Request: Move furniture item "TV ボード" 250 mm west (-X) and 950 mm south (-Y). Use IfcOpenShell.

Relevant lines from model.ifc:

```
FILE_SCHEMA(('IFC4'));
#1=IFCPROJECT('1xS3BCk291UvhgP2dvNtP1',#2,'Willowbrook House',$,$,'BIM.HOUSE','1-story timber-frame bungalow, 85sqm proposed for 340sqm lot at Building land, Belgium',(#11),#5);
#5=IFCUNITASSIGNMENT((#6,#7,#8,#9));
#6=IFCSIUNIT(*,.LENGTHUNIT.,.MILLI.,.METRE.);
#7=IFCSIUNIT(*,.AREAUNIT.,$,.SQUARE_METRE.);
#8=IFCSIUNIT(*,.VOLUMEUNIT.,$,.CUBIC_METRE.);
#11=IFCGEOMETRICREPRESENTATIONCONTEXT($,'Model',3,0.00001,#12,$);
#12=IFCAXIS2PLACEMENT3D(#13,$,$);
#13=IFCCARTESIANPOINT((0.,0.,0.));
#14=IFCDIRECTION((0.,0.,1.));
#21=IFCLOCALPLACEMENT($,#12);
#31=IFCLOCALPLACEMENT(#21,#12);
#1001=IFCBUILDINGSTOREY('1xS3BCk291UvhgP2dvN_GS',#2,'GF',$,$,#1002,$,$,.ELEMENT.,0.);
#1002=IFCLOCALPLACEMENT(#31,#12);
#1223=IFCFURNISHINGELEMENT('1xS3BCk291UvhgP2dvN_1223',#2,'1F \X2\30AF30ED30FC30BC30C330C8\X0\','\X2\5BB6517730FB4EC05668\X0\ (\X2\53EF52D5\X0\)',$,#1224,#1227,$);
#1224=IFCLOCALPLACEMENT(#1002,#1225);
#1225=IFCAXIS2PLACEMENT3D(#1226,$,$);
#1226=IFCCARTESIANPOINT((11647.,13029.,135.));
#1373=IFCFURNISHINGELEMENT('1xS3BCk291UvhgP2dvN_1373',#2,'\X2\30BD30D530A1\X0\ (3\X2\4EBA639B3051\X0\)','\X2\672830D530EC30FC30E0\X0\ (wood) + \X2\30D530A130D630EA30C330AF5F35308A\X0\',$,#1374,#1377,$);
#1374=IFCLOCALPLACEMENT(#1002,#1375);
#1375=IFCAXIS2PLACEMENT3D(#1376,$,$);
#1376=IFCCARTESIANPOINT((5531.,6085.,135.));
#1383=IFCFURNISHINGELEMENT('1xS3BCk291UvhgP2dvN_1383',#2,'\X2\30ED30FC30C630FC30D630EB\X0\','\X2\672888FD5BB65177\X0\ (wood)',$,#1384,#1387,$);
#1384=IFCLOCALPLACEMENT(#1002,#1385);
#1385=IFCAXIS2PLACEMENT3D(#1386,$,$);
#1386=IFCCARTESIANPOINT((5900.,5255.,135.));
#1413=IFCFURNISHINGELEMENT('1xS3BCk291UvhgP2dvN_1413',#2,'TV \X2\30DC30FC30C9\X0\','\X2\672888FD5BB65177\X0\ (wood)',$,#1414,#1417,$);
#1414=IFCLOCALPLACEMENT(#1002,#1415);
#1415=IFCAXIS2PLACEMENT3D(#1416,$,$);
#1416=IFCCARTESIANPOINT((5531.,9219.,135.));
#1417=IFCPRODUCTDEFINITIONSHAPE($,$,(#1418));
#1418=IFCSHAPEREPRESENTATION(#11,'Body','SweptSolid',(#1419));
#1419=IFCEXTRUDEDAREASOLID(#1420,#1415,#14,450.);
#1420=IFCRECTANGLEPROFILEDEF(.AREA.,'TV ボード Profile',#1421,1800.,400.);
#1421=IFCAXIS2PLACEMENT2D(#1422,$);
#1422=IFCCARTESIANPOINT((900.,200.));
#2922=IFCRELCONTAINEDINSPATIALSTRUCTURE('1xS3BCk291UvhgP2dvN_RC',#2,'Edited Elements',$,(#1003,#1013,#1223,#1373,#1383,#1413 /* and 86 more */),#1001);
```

```python
import ifcopenshell
import ifcopenshell.api.geometry
import ifcopenshell.util.placement

model = ifcopenshell.open("model.ifc")

item = model.by_id(1413)
matrix = ifcopenshell.util.placement.get_local_placement(item.ObjectPlacement)
matrix[0, 3] -= 250.0
matrix[1, 3] -= 950.0
ifcopenshell.api.geometry.edit_object_placement(model, product=item, matrix=matrix, is_si=False)

print(ifcopenshell.util.placement.get_local_placement(item.ObjectPlacement).round(3) + 0.0)

model.write("model_updated.ifc")
```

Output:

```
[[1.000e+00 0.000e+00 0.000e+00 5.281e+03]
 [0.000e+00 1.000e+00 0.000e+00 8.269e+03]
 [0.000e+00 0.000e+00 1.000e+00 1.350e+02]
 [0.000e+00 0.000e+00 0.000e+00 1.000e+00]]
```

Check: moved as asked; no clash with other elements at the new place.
